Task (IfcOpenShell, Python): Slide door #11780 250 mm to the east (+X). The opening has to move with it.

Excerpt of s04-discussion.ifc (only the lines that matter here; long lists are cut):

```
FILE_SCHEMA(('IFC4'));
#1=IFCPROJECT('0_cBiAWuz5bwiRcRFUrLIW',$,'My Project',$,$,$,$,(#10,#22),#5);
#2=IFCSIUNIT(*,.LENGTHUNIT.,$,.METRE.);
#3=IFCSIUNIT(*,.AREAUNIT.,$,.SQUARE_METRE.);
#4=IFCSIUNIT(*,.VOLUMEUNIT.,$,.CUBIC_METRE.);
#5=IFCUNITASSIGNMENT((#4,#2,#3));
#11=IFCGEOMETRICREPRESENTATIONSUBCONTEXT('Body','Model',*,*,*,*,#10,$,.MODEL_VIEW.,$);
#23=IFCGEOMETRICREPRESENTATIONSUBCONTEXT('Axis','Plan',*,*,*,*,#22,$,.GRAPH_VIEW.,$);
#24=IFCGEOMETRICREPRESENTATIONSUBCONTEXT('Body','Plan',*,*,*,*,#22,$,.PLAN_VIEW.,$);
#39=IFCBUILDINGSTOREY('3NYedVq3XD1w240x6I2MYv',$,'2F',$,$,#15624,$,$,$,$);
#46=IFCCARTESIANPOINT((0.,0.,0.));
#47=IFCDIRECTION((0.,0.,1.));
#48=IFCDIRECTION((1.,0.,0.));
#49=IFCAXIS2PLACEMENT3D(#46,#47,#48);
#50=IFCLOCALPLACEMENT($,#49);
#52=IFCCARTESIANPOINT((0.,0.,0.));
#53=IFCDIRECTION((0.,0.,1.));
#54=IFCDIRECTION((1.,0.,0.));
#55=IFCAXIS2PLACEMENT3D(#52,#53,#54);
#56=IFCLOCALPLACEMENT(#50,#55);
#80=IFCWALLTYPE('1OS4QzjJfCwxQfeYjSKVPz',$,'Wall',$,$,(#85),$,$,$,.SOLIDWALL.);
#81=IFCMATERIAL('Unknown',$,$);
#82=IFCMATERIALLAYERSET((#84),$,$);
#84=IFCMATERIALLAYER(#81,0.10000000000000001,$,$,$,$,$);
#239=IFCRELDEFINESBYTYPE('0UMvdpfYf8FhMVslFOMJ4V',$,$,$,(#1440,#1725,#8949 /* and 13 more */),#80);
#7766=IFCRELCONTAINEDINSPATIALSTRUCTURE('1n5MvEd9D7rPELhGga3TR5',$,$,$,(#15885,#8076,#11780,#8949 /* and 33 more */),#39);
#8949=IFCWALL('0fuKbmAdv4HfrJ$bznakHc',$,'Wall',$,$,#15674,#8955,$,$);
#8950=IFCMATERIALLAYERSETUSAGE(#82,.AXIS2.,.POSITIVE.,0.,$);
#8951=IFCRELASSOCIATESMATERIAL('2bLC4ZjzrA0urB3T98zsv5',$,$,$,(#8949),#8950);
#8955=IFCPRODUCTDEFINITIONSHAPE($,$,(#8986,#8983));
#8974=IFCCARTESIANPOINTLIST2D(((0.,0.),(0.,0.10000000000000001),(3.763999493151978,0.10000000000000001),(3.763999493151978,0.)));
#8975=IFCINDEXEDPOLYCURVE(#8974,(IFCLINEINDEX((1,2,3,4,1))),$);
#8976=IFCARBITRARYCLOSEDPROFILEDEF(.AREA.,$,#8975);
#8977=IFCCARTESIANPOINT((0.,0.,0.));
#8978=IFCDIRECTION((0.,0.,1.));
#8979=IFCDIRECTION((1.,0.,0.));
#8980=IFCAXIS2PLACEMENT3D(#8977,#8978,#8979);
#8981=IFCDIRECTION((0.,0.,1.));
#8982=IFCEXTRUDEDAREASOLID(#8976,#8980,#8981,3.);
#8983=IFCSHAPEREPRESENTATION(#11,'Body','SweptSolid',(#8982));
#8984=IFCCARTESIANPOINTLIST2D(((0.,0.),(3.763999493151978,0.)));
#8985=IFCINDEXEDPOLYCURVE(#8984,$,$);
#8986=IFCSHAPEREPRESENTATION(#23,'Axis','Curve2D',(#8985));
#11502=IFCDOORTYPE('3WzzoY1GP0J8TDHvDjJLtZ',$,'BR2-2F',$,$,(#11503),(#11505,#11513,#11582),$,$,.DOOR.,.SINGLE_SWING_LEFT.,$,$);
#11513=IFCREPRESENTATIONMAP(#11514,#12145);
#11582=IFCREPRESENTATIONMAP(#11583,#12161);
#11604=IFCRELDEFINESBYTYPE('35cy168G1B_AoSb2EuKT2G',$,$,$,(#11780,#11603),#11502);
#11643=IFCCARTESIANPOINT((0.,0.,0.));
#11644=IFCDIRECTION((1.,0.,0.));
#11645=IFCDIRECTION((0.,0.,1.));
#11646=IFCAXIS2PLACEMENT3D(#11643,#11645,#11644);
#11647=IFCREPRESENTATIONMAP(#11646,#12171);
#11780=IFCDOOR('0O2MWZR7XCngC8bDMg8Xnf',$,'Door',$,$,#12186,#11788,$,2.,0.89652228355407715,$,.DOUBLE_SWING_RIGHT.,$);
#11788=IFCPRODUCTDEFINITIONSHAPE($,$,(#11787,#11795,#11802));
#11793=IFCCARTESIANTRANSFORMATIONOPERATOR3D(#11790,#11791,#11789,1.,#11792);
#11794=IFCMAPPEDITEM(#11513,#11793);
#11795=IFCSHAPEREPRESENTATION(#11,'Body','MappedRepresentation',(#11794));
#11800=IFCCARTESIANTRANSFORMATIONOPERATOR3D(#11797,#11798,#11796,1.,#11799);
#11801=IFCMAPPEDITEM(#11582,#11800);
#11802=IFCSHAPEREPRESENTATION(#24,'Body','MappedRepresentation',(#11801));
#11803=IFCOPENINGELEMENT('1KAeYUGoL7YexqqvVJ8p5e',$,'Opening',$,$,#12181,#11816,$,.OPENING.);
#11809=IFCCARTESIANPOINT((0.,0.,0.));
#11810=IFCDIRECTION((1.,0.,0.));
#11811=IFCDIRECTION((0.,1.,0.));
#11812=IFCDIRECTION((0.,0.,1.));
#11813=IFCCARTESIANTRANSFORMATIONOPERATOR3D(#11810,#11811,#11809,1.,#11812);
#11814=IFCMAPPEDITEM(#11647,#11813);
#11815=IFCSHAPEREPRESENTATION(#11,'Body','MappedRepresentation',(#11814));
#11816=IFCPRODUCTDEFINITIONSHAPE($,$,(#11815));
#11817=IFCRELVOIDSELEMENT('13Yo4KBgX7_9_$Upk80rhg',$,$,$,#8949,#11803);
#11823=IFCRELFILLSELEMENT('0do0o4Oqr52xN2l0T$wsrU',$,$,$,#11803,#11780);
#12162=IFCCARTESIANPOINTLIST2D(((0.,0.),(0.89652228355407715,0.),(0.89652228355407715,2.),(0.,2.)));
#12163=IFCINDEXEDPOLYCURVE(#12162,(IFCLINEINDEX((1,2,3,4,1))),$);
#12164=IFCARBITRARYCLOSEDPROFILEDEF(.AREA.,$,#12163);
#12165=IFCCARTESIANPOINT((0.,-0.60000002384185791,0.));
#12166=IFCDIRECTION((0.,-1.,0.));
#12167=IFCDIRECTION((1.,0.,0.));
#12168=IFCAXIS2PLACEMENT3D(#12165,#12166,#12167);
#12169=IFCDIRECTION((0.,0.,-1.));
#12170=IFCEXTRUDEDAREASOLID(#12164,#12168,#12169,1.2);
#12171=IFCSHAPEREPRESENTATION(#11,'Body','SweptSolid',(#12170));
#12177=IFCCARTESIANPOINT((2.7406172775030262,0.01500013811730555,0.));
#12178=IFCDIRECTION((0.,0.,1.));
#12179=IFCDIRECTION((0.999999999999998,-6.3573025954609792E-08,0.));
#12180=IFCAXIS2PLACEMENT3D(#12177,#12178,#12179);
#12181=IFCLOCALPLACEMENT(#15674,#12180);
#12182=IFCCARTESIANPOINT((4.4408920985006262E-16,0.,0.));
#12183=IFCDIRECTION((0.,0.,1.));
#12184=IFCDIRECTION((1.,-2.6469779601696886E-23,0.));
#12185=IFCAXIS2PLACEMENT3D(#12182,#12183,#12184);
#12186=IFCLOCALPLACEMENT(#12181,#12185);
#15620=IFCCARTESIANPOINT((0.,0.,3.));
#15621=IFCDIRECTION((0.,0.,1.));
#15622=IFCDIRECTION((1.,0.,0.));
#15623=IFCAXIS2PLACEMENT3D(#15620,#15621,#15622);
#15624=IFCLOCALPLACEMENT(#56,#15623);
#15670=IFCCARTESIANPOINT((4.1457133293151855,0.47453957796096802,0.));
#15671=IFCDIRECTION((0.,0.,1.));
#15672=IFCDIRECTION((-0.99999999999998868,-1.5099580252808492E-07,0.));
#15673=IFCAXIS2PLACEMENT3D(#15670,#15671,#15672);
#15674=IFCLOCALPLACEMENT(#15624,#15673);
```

```python
import ifcopenshell
import ifcopenshell.api.geometry
import ifcopenshell.util.placement
import ifcopenshell.util.unit

model = ifcopenshell.open("s04-discussion.ifc")
unit_scale = ifcopenshell.util.unit.calculate_unit_scale(model)

door = model.by_guid("0O2MWZR7XCngC8bDMg8Xnf")
opening = door.FillsVoids[0].RelatingOpeningElement
wall = opening.VoidsElements[0].RelatingBuildingElement

wall_matrix = ifcopenshell.util.placement.get_local_placement(wall.ObjectPlacement)
shift = wall_matrix[:3, 0] * -0.25 / unit_scale
before = ifcopenshell.util.placement.get_local_placement(door.ObjectPlacement)[:3, 3].copy()

# The door is placed relative to its opening, so it follows when the opening moves.
matrix = ifcopenshell.util.placement.get_local_placement(opening.ObjectPlacement)
matrix[:3, 3] += shift
ifcopenshell.api.geometry.edit_object_placement(
    model, product=opening, matrix=matrix, is_si=False, should_transform_children=True
)

after = ifcopenshell.util.placement.get_local_placement(door.ObjectPlacement)[:3, 3]
print("door moved by", (after - before).round(3) + 0.0)

model.write("s04-discussion-out.ifc")
```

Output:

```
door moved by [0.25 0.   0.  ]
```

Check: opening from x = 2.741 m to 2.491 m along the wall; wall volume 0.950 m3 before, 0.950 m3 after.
